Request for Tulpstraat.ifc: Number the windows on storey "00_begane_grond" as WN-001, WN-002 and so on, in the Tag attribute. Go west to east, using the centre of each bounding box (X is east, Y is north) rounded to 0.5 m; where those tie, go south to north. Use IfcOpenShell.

First a look at what the model holds.

```python
import ifcopenshell
import ifcopenshell.util.element
import ifcopenshell.util.placement

model = ifcopenshell.open("Tulpstraat.ifc")
print(model.schema)
storey = next(s for s in model.by_type("IfcBuildingStorey") if s.Name == "00_begane_grond")
windows = [e for e in ifcopenshell.util.element.get_decomposition(storey) if e.is_a("IfcWindow")]
for e in sorted(windows, key=lambda e: e.id()):
    origin = ifcopenshell.util.placement.get_local_placement(e.ObjectPlacement)[:3, 3]
    print(e.id(), e.Tag, e.Name, origin.round(2) + 0.0, sep=" | ")
```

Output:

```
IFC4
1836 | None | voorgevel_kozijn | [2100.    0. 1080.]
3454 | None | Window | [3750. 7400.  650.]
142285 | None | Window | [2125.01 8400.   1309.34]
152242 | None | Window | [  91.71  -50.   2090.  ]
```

```python
import ifcopenshell
import ifcopenshell.geom
import ifcopenshell.util.element
import ifcopenshell.util.shape

model = ifcopenshell.open("Tulpstraat.ifc")
settings = ifcopenshell.geom.settings()
settings.set("use-world-coords", True)


def centre(element):
    shape = ifcopenshell.geom.create_shape(settings, element)
    return ifcopenshell.util.shape.get_bbox_centroid(shape.geometry)


storey = next(s for s in model.by_type("IfcBuildingStorey") if s.Name == "00_begane_grond")
windows = [e for e in ifcopenshell.util.element.get_decomposition(storey) if e.is_a("IfcWindow")]

# Insertion points can sit at a corner or the storey origin, so sort by the geometry (in metres).
centres = {e: centre(e) for e in windows}
windows.sort(key=lambda e: (round(centres[e][0] / 0.5), centres[e][1]))

for i, e in enumerate(windows, start=1):
    number = f"WN-0{i:02d}"
    e.Tag = number
    print(e.id(), number)

model.write("Tulpstraat_v2.ifc")
```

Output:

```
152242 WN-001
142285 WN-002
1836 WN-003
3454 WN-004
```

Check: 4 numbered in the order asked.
